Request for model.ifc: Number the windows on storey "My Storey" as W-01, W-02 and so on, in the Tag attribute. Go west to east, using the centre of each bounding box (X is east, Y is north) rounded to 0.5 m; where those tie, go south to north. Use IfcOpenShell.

First a look at what the model holds.

```python
import ifcopenshell
import ifcopenshell.util.element
import ifcopenshell.util.placement

model = ifcopenshell.open("model.ifc")
print(model.schema)
storey = next(s for s in model.by_type("IfcBuildingStorey") if s.Name == "My Storey")
windows = [e for e in ifcopenshell.util.element.get_decomposition(storey) if e.is_a("IfcWindow")]
for e in sorted(windows, key=lambda e: e.id()):
    origin = ifcopenshell.util.placement.get_local_placement(e.ObjectPlacement)[:3, 3]
    print(e.id(), e.Tag, e.Name, origin.round(2) + 0.0, sep=" | ")
```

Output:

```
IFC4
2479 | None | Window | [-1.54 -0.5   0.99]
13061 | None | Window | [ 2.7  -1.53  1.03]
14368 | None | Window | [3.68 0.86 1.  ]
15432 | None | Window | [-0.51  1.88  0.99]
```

```python
import ifcopenshell
import ifcopenshell.geom
import ifcopenshell.util.element
import ifcopenshell.util.shape

model = ifcopenshell.open("model.ifc")
settings = ifcopenshell.geom.settings()
settings.set("use-world-coords", True)


def centre(element):
    shape = ifcopenshell.geom.create_shape(settings, element)
    return ifcopenshell.util.shape.get_bbox_centroid(shape.geometry)


storey = next(s for s in model.by_type("IfcBuildingStorey") if s.Name == "My Storey")
windows = [e for e in ifcopenshell.util.element.get_decomposition(storey) if e.is_a("IfcWindow")]

# Insertion points can sit at a corner or the storey origin, so sort by the geometry (in metres).
centres = {e: centre(e) for e in windows}
windows.sort(key=lambda e: (round(centres[e][0] / 0.5), centres[e][1]))

for i, e in enumerate(windows, start=1):
    number = f"W-{i:02d}"
    e.Tag = number
    print(e.id(), number)

model.write("model-out.ifc")
```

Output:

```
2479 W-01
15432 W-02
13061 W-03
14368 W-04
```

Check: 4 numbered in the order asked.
